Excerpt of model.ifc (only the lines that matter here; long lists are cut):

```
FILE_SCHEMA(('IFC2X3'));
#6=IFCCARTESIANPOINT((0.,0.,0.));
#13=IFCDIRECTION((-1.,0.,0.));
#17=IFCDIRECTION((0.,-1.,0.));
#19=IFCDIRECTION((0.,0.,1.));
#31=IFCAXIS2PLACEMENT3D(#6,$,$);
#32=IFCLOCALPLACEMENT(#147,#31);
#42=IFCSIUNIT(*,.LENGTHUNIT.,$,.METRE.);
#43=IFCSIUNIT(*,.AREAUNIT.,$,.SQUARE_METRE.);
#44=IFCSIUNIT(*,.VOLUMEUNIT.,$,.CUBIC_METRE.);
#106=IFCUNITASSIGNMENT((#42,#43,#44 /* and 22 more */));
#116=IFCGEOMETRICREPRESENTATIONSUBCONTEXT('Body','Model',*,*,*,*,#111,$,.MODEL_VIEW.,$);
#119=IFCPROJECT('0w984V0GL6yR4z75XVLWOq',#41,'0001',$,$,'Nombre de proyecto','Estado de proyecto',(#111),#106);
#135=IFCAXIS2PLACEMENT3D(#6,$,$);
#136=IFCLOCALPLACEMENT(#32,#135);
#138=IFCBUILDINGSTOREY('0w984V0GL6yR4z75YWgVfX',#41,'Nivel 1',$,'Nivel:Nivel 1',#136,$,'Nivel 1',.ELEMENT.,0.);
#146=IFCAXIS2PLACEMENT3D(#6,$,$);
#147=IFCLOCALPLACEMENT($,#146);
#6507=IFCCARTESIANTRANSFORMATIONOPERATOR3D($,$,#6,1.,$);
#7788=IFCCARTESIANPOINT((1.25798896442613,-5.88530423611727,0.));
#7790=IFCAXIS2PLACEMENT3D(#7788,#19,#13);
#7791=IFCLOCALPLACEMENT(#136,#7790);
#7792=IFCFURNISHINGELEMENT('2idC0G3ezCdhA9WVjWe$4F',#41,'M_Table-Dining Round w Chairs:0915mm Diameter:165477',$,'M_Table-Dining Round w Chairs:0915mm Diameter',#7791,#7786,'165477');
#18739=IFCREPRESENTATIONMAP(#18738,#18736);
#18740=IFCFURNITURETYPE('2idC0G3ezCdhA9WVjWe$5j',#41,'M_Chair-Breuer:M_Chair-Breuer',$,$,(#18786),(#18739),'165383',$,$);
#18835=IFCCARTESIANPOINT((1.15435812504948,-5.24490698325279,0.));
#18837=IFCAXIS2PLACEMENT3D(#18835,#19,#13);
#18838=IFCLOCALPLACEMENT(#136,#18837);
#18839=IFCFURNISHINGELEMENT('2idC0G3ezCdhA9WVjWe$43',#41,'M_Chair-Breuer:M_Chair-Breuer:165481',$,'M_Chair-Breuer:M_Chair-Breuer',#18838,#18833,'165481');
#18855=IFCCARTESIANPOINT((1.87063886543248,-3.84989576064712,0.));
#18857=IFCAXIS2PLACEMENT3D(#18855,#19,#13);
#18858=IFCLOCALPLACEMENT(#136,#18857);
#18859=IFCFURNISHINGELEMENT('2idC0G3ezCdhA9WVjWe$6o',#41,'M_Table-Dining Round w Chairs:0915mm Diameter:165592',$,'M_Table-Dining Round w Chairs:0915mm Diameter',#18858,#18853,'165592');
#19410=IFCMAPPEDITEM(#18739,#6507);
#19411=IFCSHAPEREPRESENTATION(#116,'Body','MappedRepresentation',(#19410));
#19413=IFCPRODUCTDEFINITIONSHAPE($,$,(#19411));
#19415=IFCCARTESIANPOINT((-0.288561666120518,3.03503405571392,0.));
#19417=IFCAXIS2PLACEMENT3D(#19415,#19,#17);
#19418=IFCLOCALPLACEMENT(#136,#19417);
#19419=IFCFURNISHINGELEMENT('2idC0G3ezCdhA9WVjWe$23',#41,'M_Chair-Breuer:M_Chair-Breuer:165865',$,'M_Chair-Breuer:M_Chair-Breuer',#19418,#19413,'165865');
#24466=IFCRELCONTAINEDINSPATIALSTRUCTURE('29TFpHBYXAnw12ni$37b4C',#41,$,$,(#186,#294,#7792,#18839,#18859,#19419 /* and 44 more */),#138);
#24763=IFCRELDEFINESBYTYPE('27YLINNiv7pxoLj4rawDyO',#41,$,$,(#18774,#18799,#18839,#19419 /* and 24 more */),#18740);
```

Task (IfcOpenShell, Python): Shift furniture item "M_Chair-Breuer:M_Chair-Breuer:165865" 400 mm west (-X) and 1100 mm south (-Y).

```python
import ifcopenshell
import ifcopenshell.api.geometry
import ifcopenshell.util.placement
import ifcopenshell.util.unit

model = ifcopenshell.open("model.ifc")
unit_scale = ifcopenshell.util.unit.calculate_unit_scale(model)

item = model.by_guid("2idC0G3ezCdhA9WVjWe$23")
matrix = ifcopenshell.util.placement.get_local_placement(item.ObjectPlacement)
matrix[0, 3] -= 0.4 / unit_scale
matrix[1, 3] -= 1.1 / unit_scale
ifcopenshell.api.geometry.edit_object_placement(model, product=item, matrix=matrix, is_si=False)

print(ifcopenshell.util.placement.get_local_placement(item.ObjectPlacement).round(3) + 0.0)

model.write("model_rev.ifc")
```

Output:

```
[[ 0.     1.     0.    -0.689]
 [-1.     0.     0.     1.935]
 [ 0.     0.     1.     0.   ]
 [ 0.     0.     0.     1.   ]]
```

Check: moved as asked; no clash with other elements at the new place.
